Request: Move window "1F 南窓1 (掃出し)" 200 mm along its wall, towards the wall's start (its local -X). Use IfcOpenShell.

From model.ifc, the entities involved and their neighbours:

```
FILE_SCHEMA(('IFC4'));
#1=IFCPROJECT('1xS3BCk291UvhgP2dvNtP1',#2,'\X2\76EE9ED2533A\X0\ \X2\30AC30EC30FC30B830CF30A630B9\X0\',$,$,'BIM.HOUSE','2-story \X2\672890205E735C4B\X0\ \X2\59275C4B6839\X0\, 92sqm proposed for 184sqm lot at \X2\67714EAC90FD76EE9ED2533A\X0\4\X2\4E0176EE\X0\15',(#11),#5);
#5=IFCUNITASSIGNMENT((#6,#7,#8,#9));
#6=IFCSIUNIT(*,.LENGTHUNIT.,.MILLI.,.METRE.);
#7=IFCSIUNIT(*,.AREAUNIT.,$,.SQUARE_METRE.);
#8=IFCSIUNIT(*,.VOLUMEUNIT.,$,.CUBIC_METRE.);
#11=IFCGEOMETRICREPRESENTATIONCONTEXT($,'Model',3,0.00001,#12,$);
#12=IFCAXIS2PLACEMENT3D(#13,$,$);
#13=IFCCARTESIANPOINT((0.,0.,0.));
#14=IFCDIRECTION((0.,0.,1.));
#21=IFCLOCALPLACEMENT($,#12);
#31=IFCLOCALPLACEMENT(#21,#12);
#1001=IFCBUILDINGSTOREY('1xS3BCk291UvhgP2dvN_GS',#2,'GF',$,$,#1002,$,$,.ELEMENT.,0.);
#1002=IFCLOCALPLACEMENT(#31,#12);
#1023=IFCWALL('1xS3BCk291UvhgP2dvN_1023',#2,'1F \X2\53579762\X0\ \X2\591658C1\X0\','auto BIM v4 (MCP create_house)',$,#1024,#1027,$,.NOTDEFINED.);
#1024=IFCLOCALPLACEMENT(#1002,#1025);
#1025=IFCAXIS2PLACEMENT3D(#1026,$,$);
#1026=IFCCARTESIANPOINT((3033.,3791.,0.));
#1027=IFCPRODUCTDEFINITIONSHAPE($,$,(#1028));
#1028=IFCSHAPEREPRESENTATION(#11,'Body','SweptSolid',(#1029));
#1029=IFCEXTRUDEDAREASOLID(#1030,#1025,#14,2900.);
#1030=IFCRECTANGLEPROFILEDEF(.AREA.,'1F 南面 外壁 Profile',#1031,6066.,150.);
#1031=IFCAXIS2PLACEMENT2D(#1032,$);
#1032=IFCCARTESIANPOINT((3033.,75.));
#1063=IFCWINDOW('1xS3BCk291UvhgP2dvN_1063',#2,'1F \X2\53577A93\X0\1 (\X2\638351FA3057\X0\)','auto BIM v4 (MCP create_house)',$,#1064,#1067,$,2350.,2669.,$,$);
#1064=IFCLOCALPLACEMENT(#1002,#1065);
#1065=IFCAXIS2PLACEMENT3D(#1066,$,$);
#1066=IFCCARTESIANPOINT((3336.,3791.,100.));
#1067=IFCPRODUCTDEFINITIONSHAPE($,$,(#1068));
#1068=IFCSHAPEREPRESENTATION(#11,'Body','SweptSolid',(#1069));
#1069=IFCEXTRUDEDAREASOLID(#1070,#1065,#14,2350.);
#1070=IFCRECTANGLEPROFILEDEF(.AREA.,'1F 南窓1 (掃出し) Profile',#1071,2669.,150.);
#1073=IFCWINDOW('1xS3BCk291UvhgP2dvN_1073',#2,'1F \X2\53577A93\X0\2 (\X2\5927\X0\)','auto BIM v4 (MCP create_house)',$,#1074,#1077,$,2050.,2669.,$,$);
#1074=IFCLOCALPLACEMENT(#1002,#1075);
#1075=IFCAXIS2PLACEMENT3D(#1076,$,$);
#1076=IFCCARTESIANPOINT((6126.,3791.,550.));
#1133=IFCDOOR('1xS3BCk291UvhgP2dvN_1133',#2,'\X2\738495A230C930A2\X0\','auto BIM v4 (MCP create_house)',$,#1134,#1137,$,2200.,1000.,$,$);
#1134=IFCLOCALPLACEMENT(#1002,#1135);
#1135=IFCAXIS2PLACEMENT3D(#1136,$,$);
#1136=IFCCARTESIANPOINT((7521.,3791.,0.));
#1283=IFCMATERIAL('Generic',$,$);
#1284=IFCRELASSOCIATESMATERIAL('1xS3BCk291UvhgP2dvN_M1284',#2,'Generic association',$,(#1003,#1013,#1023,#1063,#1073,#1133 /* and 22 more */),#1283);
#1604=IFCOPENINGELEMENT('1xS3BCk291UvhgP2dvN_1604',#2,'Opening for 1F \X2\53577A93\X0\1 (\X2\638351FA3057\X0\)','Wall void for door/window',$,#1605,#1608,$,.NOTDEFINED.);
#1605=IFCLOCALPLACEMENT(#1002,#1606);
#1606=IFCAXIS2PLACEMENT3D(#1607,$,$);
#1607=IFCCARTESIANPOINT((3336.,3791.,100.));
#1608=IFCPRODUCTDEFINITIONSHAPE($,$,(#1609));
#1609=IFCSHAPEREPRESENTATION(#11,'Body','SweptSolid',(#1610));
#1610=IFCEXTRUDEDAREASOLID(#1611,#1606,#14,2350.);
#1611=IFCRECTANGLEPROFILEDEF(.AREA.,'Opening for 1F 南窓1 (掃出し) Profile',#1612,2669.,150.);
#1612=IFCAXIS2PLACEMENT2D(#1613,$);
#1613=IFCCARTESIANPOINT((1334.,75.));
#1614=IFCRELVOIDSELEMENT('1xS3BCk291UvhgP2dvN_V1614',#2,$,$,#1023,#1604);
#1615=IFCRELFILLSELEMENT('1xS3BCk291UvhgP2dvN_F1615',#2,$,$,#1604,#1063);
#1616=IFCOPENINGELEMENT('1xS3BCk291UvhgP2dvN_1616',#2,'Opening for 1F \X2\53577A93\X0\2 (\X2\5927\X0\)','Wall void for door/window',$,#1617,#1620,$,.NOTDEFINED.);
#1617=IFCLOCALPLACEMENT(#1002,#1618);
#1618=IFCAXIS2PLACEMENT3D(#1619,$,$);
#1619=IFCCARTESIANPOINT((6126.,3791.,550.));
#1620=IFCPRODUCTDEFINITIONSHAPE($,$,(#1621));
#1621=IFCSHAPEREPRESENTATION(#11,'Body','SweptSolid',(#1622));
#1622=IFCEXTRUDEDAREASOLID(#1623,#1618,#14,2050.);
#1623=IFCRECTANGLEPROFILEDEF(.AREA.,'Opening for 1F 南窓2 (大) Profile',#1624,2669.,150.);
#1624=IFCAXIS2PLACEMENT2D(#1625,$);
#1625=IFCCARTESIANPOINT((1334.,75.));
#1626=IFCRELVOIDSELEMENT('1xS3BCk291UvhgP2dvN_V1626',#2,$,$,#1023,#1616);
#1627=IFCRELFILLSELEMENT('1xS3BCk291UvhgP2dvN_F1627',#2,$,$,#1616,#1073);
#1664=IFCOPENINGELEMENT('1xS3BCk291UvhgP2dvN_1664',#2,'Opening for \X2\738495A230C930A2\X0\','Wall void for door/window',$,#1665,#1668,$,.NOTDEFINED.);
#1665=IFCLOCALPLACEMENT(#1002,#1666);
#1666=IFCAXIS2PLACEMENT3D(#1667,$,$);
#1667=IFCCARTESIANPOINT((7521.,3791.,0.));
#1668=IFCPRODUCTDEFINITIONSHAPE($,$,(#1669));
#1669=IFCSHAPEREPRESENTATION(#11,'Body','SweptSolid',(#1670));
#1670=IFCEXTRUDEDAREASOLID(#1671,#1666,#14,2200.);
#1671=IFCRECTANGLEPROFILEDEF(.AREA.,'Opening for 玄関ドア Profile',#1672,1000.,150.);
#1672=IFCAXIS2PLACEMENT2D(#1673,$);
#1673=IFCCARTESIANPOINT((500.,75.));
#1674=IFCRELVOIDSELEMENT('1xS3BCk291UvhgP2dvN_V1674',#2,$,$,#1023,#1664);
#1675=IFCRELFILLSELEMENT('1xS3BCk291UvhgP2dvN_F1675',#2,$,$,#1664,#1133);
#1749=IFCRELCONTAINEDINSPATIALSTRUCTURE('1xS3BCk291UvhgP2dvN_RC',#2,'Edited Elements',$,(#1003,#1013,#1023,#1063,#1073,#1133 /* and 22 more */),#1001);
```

```python
import ifcopenshell
import ifcopenshell.api.geometry
import ifcopenshell.util.placement
import ifcopenshell.util.unit

model = ifcopenshell.open("model.ifc")
unit_scale = ifcopenshell.util.unit.calculate_unit_scale(model)

window = model.by_guid("1xS3BCk291UvhgP2dvN_1063")
opening = window.FillsVoids[0].RelatingOpeningElement
wall = opening.VoidsElements[0].RelatingBuildingElement

wall_matrix = ifcopenshell.util.placement.get_local_placement(wall.ObjectPlacement)
shift = wall_matrix[:3, 0] * -0.2 / unit_scale
before = ifcopenshell.util.placement.get_local_placement(window.ObjectPlacement)[:3, 3].copy()

# The window is not placed relative to its opening, so move both.
for product in (opening, window):
    matrix = ifcopenshell.util.placement.get_local_placement(product.ObjectPlacement)
    matrix[:3, 3] += shift
    ifcopenshell.api.geometry.edit_object_placement(model, product=product, matrix=matrix, is_si=False)

after = ifcopenshell.util.placement.get_local_placement(window.ObjectPlacement)[:3, 3]
print("window moved by", (after - before).round(3) + 0.0)

model.write("model_updated.ifc")
```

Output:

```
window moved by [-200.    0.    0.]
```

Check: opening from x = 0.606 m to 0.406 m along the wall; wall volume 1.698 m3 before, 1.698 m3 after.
